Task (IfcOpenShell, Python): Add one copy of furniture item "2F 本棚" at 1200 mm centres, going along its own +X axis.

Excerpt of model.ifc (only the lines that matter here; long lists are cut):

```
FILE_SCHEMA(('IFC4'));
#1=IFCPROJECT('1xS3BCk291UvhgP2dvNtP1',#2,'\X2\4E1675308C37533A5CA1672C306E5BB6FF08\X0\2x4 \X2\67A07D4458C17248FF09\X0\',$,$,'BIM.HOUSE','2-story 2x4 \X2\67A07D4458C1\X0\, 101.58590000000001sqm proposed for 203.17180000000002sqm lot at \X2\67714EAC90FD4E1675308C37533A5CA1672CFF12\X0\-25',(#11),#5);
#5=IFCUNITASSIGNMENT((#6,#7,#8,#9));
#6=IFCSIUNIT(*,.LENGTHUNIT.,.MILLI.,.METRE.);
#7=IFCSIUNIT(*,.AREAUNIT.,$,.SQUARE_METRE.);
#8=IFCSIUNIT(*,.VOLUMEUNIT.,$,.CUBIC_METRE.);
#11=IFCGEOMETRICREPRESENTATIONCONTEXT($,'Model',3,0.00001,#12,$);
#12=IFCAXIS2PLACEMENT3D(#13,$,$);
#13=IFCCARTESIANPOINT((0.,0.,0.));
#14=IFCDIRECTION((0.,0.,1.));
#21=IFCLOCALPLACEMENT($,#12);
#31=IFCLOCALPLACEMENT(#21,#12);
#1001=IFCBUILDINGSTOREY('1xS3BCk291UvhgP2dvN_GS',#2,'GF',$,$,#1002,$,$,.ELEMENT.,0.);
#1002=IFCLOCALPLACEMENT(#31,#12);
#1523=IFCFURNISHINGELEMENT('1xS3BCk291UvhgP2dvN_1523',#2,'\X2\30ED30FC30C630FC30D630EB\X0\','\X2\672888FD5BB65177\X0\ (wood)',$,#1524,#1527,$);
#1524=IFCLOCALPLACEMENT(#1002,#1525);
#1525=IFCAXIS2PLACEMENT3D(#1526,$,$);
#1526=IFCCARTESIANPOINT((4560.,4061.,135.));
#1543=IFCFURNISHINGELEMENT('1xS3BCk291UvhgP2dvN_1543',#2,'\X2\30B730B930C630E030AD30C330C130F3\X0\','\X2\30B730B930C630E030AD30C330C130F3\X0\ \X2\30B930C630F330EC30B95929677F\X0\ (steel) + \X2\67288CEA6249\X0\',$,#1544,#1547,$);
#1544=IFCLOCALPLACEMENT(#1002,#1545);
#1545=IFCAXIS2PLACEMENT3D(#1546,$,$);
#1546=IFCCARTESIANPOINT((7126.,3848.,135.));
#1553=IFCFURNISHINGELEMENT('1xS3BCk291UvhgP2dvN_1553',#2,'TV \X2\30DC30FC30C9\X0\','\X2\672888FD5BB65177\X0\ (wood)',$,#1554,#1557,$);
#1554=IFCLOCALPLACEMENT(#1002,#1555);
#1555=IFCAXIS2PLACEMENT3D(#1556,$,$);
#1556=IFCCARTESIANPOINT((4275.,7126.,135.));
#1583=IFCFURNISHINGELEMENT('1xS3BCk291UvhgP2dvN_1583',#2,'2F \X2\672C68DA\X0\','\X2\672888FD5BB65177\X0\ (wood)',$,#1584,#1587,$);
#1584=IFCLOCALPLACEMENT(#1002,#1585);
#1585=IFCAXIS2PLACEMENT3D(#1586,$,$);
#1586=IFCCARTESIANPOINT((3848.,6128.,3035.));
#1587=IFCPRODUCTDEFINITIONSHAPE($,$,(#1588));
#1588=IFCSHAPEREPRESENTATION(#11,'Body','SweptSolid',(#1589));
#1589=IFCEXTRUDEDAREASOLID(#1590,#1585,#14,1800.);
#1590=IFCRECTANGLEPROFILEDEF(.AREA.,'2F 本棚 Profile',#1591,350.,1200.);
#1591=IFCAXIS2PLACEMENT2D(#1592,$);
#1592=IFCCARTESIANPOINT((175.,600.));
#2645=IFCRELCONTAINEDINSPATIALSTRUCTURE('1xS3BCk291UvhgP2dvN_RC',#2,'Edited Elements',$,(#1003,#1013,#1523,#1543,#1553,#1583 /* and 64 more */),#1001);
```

```python
import ifcopenshell
import ifcopenshell.api.geometry
import ifcopenshell.api.root
import ifcopenshell.util.element
import ifcopenshell.util.placement

model = ifcopenshell.open("model.ifc")


def reuse_history(source, copy):
    """copy_class also copies each property set's owner history, people and application; keep the originals."""
    for rel in copy.IsDefinedBy:
        if rel.is_a("IfcRelDefinesByProperties") and (history := rel.RelatingPropertyDefinition.OwnerHistory):
            rel.RelatingPropertyDefinition.OwnerHistory = source.OwnerHistory
            ifcopenshell.util.element.remove_deep2(model, history)


source = model.by_guid("1xS3BCk291UvhgP2dvN_1583")
base = ifcopenshell.util.placement.get_local_placement(source.ObjectPlacement)
step = base[:3, 0] * 1200.0

for i in range(1, 2):
    copy = ifcopenshell.api.root.copy_class(model, product=source)
    copy.Representation = ifcopenshell.util.element.copy_deep(
        model, source.Representation, exclude=["IfcGeometricRepresentationContext", "IfcRepresentationMap"]
    )
    reuse_history(source, copy)
    matrix = base.copy()
    matrix[:3, 3] += i * step
    print("added at", matrix[:3, 3].round(3) + 0.0)
    ifcopenshell.api.geometry.edit_object_placement(model, product=copy, matrix=matrix, is_si=False)

model.write("model_updated.ifc")
```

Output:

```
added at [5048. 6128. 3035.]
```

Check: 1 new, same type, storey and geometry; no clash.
